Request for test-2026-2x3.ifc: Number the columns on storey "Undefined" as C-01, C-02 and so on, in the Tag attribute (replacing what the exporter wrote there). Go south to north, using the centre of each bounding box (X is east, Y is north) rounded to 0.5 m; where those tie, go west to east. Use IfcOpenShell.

First a look at what the model holds.

```python
import ifcopenshell
import ifcopenshell.util.element
import ifcopenshell.util.placement

model = ifcopenshell.open("test-2026-2x3.ifc")
print(model.schema)
storey = next(s for s in model.by_type("IfcBuildingStorey") if s.Name == "Undefined")
columns = [e for e in ifcopenshell.util.element.get_decomposition(storey) if e.is_a("IfcColumn")]
for e in sorted(columns, key=lambda e: e.id()):
    origin = ifcopenshell.util.placement.get_local_placement(e.ObjectPlacement)[:3, 3]
    print(e.id(), e.Tag, e.Name, origin.round(2) + 0.0, sep=" | ")
```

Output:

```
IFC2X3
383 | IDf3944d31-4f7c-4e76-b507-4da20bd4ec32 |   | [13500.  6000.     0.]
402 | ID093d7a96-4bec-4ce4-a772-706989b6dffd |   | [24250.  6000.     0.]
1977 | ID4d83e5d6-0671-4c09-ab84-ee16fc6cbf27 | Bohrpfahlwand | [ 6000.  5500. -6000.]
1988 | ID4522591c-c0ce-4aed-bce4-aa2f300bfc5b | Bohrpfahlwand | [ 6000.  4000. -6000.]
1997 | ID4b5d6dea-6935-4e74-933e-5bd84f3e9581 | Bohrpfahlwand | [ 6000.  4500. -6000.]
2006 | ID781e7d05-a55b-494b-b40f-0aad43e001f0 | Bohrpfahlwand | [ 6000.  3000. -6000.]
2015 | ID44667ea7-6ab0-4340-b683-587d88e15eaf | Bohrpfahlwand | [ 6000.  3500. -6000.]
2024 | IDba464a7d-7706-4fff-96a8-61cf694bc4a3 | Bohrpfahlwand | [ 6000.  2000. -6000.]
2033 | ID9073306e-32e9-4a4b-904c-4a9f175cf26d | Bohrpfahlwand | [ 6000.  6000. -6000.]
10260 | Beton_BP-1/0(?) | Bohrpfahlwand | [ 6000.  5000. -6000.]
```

```python
import ifcopenshell
import ifcopenshell.geom
import ifcopenshell.util.element
import ifcopenshell.util.shape

model = ifcopenshell.open("test-2026-2x3.ifc")
settings = ifcopenshell.geom.settings()
settings.set("use-world-coords", True)


def centre(element):
    shape = ifcopenshell.geom.create_shape(settings, element)
    return ifcopenshell.util.shape.get_bbox_centroid(shape.geometry)


storey = next(s for s in model.by_type("IfcBuildingStorey") if s.Name == "Undefined")
columns = [e for e in ifcopenshell.util.element.get_decomposition(storey) if e.is_a("IfcColumn")]

# Insertion points can sit at a corner or the storey origin, so sort by the geometry (in metres).
centres = {e: centre(e) for e in columns}
columns.sort(key=lambda e: (round(centres[e][1] / 0.5), centres[e][0]))

for i, e in enumerate(columns, start=1):
    number = f"C-{i:02d}"
    e.Tag = number
    print(e.id(), number)

model.write("test-2026-2x3_edited.ifc")
```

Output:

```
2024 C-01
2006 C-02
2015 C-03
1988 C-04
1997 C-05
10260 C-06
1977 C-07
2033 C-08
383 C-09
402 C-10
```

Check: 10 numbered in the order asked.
